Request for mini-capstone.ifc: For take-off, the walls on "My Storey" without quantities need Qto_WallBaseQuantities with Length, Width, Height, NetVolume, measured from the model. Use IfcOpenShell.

First a look at what the model holds.

```python
import ifcopenshell
import ifcopenshell.util.element
import ifcopenshell.util.unit

model = ifcopenshell.open("mini-capstone.ifc")
print(model.schema)
for unit_type in ("LENGTHUNIT", "AREAUNIT", "VOLUMEUNIT"):
    print(unit_type, ifcopenshell.util.unit.calculate_unit_scale(model, unit_type))
storey = next(s for s in model.by_type("IfcBuildingStorey") if s.Name == "My Storey")
walls = [e for e in ifcopenshell.util.element.get_decomposition(storey) if e.is_a("IfcWall")]
for e in sorted(walls, key=lambda e: e.id()):
    print(e.id(), e.is_a(), e.Name, list(ifcopenshell.util.element.get_psets(e, qtos_only=True)), sep=" | ")
```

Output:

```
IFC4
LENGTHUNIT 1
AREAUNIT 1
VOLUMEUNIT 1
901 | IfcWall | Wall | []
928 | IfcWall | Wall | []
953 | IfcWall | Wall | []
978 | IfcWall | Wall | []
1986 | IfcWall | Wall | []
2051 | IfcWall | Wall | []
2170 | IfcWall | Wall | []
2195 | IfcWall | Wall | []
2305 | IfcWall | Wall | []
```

```python
import ifcopenshell
import ifcopenshell.api.pset
import ifcopenshell.geom
import ifcopenshell.util.element
import ifcopenshell.util.shape
import ifcopenshell.util.unit

model = ifcopenshell.open("mini-capstone.ifc")
unit_scale = ifcopenshell.util.unit.calculate_unit_scale(model)
volume_scale = ifcopenshell.util.unit.calculate_unit_scale(model, "VOLUMEUNIT")
settings = ifcopenshell.geom.settings()

storey = next(s for s in model.by_type("IfcBuildingStorey") if s.Name == "My Storey")
walls = [e for e in ifcopenshell.util.element.get_decomposition(storey) if e.is_a("IfcWall")]

for e in sorted(walls, key=lambda e: e.id()):
    if ifcopenshell.util.element.get_psets(e, qtos_only=True, should_inherit=False):
        continue
    # Geometry comes back in metres, in the element's own axes.
    shape = ifcopenshell.geom.create_shape(settings, e)
    values = {
        "Length": ifcopenshell.util.shape.get_x(shape.geometry) / unit_scale,
        "Width": ifcopenshell.util.shape.get_y(shape.geometry) / unit_scale,
        "Height": ifcopenshell.util.shape.get_z(shape.geometry) / unit_scale,
        "NetVolume": ifcopenshell.util.shape.get_volume(shape.geometry) / volume_scale,
    }
    qto = ifcopenshell.api.pset.add_qto(model, product=e, name="Qto_WallBaseQuantities")
    ifcopenshell.api.pset.edit_qto(model, qto=qto, properties=values)
    print(e.id(), {k: round(v, 3) for k, v in values.items()})

model.write("mini-capstone_edited.ifc")
```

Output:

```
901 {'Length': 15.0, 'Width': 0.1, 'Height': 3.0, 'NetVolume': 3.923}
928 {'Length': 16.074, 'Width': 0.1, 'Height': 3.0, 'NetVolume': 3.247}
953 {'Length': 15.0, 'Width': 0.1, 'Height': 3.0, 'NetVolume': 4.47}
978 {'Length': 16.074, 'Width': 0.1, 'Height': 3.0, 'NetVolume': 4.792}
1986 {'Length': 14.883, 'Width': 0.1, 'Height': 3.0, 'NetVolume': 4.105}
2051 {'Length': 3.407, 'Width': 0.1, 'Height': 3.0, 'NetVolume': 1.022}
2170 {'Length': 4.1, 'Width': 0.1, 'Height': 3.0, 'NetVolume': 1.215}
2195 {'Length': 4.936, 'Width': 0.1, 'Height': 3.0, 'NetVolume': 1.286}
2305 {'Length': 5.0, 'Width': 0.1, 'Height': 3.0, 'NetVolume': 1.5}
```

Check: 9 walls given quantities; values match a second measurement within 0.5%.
